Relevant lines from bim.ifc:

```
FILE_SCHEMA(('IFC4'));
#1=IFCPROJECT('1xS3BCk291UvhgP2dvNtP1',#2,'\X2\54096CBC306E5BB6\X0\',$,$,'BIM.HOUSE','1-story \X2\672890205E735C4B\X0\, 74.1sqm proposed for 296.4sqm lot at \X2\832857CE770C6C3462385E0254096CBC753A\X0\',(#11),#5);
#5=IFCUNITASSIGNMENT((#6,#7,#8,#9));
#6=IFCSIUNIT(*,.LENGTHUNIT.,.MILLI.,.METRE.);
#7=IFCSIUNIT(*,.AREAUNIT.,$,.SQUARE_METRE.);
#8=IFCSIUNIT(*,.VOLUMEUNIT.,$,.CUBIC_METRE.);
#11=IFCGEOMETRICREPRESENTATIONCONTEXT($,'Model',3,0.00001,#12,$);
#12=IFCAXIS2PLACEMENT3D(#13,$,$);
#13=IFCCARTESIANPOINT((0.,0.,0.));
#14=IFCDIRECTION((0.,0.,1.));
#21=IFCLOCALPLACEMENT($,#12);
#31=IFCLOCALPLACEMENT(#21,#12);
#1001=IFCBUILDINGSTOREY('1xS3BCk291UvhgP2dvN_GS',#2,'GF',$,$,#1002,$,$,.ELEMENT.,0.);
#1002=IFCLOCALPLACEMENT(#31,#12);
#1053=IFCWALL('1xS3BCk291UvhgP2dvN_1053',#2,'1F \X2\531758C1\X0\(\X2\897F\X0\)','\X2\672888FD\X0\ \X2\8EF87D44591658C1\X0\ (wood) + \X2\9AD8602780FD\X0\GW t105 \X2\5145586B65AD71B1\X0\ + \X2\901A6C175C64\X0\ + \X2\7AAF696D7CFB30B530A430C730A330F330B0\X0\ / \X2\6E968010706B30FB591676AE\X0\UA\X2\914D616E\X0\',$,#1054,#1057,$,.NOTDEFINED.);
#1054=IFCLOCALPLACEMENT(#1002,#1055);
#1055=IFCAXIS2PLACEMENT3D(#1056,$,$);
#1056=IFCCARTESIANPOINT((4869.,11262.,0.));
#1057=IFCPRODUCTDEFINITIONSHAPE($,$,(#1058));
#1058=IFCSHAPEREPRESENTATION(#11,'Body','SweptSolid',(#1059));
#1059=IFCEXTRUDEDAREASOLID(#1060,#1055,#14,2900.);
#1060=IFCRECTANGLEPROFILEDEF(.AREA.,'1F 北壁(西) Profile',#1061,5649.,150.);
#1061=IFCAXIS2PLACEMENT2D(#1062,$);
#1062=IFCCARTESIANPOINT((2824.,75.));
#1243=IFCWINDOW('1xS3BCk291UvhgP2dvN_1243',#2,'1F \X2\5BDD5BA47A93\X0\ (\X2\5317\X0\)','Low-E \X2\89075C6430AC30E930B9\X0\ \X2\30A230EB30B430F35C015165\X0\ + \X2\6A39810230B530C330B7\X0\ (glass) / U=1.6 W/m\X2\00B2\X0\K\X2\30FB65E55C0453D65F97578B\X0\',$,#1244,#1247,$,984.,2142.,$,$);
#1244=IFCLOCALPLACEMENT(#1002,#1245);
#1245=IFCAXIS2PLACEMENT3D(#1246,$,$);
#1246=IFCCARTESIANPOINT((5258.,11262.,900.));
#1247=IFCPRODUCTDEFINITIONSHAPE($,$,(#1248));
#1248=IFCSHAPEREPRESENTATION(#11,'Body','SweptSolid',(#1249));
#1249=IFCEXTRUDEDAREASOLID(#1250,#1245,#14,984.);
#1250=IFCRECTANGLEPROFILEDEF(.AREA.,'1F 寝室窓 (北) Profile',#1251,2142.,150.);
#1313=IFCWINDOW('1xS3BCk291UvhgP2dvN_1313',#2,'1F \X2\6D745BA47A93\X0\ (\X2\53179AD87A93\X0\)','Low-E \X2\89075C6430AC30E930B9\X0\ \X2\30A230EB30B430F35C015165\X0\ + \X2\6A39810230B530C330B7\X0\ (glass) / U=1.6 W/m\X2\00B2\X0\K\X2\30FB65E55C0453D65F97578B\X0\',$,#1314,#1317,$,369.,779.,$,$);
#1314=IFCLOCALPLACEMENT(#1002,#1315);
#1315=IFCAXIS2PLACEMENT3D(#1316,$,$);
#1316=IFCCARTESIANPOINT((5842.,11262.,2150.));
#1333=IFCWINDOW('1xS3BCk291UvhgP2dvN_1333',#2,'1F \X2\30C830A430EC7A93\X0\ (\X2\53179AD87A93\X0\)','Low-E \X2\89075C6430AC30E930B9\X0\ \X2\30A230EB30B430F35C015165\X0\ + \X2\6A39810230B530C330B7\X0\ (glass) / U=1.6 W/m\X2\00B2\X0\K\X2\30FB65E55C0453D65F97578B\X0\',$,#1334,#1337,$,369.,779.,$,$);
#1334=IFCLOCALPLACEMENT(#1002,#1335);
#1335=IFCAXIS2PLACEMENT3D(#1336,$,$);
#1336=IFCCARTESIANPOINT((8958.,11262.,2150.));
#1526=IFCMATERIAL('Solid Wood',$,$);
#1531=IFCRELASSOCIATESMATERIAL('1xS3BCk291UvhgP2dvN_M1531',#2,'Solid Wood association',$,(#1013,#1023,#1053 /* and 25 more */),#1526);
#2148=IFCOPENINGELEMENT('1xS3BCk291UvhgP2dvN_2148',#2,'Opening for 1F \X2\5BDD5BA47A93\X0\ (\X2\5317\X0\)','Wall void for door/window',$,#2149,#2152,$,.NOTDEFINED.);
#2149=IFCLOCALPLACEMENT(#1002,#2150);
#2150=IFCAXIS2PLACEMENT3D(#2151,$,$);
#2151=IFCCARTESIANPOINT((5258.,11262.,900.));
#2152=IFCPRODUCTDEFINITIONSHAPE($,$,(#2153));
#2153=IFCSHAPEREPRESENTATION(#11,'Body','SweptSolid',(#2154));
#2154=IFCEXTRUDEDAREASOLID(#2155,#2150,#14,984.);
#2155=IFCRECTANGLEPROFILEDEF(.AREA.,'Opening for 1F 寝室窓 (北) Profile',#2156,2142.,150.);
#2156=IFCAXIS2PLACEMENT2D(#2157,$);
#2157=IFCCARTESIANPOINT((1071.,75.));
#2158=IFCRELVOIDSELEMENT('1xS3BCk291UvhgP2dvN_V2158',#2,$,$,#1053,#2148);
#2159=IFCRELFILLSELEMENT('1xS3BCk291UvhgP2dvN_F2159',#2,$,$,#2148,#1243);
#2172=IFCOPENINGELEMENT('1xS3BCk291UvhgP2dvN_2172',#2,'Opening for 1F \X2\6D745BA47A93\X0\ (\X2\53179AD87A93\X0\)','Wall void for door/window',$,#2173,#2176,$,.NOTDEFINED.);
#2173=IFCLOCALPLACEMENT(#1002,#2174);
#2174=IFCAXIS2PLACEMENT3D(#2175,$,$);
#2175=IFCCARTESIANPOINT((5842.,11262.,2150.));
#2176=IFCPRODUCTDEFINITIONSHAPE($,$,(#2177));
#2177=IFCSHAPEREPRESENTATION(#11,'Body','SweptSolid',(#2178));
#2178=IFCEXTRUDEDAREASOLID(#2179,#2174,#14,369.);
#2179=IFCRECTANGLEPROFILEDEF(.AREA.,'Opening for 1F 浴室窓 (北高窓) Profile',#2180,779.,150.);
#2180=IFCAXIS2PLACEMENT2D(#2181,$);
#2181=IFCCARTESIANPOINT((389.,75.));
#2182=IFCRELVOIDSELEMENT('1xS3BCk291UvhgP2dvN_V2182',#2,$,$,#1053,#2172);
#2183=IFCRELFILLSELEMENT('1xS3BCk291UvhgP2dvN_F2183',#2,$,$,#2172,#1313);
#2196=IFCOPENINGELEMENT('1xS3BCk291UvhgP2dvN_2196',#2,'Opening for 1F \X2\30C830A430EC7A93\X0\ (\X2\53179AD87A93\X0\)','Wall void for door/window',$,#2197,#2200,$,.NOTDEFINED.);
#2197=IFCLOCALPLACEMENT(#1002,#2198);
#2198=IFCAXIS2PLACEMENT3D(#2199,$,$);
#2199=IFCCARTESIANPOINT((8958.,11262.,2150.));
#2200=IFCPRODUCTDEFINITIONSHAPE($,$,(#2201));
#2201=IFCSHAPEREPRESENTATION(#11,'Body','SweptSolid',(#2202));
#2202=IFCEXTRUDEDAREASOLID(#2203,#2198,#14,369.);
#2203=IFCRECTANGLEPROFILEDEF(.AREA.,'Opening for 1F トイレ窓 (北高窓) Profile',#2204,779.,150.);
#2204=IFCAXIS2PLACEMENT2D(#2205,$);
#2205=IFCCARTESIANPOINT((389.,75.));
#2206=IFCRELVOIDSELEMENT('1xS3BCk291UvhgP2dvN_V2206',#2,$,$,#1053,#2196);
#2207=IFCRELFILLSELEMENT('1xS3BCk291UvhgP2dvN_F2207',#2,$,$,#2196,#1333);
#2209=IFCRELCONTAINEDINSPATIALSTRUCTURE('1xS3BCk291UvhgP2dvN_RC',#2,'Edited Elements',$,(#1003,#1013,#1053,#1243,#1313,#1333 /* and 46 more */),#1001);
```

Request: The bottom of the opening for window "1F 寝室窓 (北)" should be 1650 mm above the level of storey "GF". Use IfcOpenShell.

```python
import numpy as np
import ifcopenshell
import ifcopenshell.api.geometry
import ifcopenshell.geom
import ifcopenshell.util.element
import ifcopenshell.util.placement
import ifcopenshell.util.shape
import ifcopenshell.util.unit

model = ifcopenshell.open("bim.ifc")
unit_scale = ifcopenshell.util.unit.calculate_unit_scale(model)

window = model.by_guid("1xS3BCk291UvhgP2dvN_1243")
opening = window.FillsVoids[0].RelatingOpeningElement
storey = ifcopenshell.util.element.get_container(window, ifc_class="IfcBuildingStorey")
level = ifcopenshell.util.placement.get_local_placement(storey.ObjectPlacement)[2, 3]

# The opening's origin need not be at the sill, so measure its lowest point.
shape = ifcopenshell.geom.create_shape(ifcopenshell.geom.settings(), opening)
bottom = ifcopenshell.util.shape.get_shape_bottom_elevation(shape, shape.geometry) / unit_scale
dz = level + 1.65 / unit_scale - bottom

shift = np.array([0.0, 0.0, dz])
# The window is not placed relative to its opening, so move both.
for product in (opening, window):
    matrix = ifcopenshell.util.placement.get_local_placement(product.ObjectPlacement)
    matrix[:3, 3] += shift
    ifcopenshell.api.geometry.edit_object_placement(model, product=product, matrix=matrix, is_si=False)

print(f"moved by {dz * unit_scale:+.3f} m")

model.write("bim_edited.ifc")
```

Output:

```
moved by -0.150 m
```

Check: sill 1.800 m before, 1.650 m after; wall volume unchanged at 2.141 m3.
